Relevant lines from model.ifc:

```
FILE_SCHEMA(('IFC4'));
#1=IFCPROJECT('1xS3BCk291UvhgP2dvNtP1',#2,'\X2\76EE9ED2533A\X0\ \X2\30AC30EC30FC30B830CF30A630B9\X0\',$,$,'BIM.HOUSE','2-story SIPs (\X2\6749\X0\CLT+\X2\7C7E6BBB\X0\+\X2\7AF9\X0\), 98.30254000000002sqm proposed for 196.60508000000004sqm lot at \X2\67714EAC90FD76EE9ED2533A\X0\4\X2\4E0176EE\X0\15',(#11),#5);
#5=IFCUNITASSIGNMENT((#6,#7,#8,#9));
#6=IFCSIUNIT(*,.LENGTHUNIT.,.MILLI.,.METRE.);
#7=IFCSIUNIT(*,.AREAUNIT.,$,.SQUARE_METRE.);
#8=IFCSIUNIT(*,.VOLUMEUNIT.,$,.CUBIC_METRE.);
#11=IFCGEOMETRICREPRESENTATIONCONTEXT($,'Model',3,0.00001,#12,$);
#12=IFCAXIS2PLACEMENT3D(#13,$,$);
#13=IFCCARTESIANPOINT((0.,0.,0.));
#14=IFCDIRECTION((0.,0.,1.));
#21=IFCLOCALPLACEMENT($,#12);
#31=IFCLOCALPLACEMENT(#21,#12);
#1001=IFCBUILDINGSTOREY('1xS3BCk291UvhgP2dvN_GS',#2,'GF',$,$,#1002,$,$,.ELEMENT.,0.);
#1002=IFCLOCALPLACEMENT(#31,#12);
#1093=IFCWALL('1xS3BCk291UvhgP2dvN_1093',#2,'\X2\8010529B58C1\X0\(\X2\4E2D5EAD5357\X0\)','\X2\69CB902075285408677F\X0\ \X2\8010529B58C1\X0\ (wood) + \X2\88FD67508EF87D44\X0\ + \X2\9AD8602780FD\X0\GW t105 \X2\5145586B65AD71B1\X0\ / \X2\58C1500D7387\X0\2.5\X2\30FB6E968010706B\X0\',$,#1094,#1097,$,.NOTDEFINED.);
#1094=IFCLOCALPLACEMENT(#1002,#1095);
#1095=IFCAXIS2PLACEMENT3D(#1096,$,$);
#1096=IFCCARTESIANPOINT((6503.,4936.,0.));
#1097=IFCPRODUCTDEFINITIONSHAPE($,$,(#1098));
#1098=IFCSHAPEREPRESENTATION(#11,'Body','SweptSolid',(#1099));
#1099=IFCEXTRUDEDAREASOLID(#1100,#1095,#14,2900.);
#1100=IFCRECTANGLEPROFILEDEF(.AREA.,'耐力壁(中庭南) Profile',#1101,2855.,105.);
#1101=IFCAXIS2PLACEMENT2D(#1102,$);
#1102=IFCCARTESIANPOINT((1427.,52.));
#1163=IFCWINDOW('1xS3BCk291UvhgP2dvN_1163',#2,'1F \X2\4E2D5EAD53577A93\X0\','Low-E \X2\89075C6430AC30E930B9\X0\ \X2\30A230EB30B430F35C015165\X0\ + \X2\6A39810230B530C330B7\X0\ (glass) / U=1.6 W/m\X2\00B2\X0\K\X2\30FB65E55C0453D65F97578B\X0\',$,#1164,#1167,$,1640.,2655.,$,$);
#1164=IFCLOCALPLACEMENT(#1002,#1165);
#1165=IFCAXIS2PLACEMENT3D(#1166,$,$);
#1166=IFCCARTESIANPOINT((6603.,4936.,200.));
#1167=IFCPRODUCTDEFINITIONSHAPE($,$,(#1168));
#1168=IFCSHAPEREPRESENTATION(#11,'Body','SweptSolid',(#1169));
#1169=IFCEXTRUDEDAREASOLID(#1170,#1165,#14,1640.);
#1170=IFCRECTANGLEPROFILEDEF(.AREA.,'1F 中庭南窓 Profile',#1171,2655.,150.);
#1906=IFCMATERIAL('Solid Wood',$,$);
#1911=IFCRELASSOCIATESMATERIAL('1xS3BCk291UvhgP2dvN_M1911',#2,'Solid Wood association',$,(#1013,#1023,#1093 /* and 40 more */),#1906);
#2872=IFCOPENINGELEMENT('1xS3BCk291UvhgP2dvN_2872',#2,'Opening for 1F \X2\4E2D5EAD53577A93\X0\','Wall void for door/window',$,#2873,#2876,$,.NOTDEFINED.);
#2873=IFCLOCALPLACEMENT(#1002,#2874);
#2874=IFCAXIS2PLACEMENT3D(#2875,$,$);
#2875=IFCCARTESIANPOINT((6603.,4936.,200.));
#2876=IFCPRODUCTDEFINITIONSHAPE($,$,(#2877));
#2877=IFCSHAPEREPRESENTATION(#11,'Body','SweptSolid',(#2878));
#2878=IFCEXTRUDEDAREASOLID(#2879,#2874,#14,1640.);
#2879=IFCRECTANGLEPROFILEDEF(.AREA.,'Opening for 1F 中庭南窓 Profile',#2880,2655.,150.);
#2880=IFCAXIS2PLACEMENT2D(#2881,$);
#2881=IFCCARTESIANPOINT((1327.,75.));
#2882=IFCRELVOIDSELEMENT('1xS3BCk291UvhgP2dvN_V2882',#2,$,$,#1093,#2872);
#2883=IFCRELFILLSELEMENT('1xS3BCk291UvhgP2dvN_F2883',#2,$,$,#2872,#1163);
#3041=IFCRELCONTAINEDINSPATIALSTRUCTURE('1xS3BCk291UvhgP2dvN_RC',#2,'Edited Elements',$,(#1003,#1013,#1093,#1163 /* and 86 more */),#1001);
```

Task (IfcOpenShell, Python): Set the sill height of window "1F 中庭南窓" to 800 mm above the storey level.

```python
import numpy as np
import ifcopenshell
import ifcopenshell.api.geometry
import ifcopenshell.geom
import ifcopenshell.util.element
import ifcopenshell.util.placement
import ifcopenshell.util.shape
import ifcopenshell.util.unit

model = ifcopenshell.open("model.ifc")
unit_scale = ifcopenshell.util.unit.calculate_unit_scale(model)

window = model.by_guid("1xS3BCk291UvhgP2dvN_1163")
opening = window.FillsVoids[0].RelatingOpeningElement
storey = ifcopenshell.util.element.get_container(window, ifc_class="IfcBuildingStorey")
level = ifcopenshell.util.placement.get_local_placement(storey.ObjectPlacement)[2, 3]

# The opening's origin need not be at the sill, so measure its lowest point.
shape = ifcopenshell.geom.create_shape(ifcopenshell.geom.settings(), opening)
bottom = ifcopenshell.util.shape.get_shape_bottom_elevation(shape, shape.geometry) / unit_scale
dz = level + 0.8 / unit_scale - bottom

shift = np.array([0.0, 0.0, dz])
# The window is not placed relative to its opening, so move both.
for product in (opening, window):
    matrix = ifcopenshell.util.placement.get_local_placement(product.ObjectPlacement)
    matrix[:3, 3] += shift
    ifcopenshell.api.geometry.edit_object_placement(model, product=product, matrix=matrix, is_si=False)

print(f"moved by {dz * unit_scale:+.3f} m")

model.write("model-out.ifc")
```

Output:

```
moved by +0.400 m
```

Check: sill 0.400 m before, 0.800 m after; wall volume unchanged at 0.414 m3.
